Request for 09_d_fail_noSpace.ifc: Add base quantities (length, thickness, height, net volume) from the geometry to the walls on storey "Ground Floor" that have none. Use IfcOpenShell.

First a look at what the model holds.

```python
import ifcopenshell
import ifcopenshell.util.element
import ifcopenshell.util.unit

model = ifcopenshell.open("09_d_fail_noSpace.ifc")
print(model.schema)
for unit_type in ("LENGTHUNIT", "AREAUNIT", "VOLUMEUNIT"):
    print(unit_type, ifcopenshell.util.unit.calculate_unit_scale(model, unit_type))
storey = next(s for s in model.by_type("IfcBuildingStorey") if s.Name == "Ground Floor")
walls = [e for e in ifcopenshell.util.element.get_decomposition(storey) if e.is_a("IfcWall")]
for e in sorted(walls, key=lambda e: e.id()):
    print(e.id(), e.is_a(), e.Name, list(ifcopenshell.util.element.get_psets(e, qtos_only=True)), sep=" | ")
```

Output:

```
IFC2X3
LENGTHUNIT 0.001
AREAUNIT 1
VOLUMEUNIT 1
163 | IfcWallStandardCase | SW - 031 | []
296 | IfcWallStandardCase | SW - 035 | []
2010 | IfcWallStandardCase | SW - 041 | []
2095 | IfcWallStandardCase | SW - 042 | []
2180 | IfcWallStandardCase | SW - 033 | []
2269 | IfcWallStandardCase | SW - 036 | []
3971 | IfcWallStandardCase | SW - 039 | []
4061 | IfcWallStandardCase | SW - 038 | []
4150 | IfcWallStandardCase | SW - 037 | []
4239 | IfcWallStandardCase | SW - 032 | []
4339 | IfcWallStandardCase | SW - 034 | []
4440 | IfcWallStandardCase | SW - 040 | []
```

```python
import ifcopenshell
import ifcopenshell.api.pset
import ifcopenshell.geom
import ifcopenshell.util.element
import ifcopenshell.util.shape
import ifcopenshell.util.unit

model = ifcopenshell.open("09_d_fail_noSpace.ifc")
unit_scale = ifcopenshell.util.unit.calculate_unit_scale(model)
volume_scale = ifcopenshell.util.unit.calculate_unit_scale(model, "VOLUMEUNIT")
settings = ifcopenshell.geom.settings()

storey = next(s for s in model.by_type("IfcBuildingStorey") if s.Name == "Ground Floor")
walls = [e for e in ifcopenshell.util.element.get_decomposition(storey) if e.is_a("IfcWall")]

for e in sorted(walls, key=lambda e: e.id()):
    if ifcopenshell.util.element.get_psets(e, qtos_only=True, should_inherit=False):
        continue
    # Geometry comes back in metres, in the element's own axes.
    shape = ifcopenshell.geom.create_shape(settings, e)
    values = {
        "Length": ifcopenshell.util.shape.get_x(shape.geometry) / unit_scale,
        "Width": ifcopenshell.util.shape.get_y(shape.geometry) / unit_scale,
        "Height": ifcopenshell.util.shape.get_z(shape.geometry) / unit_scale,
        "NetVolume": ifcopenshell.util.shape.get_volume(shape.geometry) / volume_scale,
    }
    qto = ifcopenshell.api.pset.add_qto(model, product=e, name="BaseQuantities")
    ifcopenshell.api.pset.edit_qto(model, qto=qto, properties=values)
    print(e.id(), {k: round(v, 3) for k, v in values.items()})

model.write("09_d_fail_noSpace_edited.ifc")
```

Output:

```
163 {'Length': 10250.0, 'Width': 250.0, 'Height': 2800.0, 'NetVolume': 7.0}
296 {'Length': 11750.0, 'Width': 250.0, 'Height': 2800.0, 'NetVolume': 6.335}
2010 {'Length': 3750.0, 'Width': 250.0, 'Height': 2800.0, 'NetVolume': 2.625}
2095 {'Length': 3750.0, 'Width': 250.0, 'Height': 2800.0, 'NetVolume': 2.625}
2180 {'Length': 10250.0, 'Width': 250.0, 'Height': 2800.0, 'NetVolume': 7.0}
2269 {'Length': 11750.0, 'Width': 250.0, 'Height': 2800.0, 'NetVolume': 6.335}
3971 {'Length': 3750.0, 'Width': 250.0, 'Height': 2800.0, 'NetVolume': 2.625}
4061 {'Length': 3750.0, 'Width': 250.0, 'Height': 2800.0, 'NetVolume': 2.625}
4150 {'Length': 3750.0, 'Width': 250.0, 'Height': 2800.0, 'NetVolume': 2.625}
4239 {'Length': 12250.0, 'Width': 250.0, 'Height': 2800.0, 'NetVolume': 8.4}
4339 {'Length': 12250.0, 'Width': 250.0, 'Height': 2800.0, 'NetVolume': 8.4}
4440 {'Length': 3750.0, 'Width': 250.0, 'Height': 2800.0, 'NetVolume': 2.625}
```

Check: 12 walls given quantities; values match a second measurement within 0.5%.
